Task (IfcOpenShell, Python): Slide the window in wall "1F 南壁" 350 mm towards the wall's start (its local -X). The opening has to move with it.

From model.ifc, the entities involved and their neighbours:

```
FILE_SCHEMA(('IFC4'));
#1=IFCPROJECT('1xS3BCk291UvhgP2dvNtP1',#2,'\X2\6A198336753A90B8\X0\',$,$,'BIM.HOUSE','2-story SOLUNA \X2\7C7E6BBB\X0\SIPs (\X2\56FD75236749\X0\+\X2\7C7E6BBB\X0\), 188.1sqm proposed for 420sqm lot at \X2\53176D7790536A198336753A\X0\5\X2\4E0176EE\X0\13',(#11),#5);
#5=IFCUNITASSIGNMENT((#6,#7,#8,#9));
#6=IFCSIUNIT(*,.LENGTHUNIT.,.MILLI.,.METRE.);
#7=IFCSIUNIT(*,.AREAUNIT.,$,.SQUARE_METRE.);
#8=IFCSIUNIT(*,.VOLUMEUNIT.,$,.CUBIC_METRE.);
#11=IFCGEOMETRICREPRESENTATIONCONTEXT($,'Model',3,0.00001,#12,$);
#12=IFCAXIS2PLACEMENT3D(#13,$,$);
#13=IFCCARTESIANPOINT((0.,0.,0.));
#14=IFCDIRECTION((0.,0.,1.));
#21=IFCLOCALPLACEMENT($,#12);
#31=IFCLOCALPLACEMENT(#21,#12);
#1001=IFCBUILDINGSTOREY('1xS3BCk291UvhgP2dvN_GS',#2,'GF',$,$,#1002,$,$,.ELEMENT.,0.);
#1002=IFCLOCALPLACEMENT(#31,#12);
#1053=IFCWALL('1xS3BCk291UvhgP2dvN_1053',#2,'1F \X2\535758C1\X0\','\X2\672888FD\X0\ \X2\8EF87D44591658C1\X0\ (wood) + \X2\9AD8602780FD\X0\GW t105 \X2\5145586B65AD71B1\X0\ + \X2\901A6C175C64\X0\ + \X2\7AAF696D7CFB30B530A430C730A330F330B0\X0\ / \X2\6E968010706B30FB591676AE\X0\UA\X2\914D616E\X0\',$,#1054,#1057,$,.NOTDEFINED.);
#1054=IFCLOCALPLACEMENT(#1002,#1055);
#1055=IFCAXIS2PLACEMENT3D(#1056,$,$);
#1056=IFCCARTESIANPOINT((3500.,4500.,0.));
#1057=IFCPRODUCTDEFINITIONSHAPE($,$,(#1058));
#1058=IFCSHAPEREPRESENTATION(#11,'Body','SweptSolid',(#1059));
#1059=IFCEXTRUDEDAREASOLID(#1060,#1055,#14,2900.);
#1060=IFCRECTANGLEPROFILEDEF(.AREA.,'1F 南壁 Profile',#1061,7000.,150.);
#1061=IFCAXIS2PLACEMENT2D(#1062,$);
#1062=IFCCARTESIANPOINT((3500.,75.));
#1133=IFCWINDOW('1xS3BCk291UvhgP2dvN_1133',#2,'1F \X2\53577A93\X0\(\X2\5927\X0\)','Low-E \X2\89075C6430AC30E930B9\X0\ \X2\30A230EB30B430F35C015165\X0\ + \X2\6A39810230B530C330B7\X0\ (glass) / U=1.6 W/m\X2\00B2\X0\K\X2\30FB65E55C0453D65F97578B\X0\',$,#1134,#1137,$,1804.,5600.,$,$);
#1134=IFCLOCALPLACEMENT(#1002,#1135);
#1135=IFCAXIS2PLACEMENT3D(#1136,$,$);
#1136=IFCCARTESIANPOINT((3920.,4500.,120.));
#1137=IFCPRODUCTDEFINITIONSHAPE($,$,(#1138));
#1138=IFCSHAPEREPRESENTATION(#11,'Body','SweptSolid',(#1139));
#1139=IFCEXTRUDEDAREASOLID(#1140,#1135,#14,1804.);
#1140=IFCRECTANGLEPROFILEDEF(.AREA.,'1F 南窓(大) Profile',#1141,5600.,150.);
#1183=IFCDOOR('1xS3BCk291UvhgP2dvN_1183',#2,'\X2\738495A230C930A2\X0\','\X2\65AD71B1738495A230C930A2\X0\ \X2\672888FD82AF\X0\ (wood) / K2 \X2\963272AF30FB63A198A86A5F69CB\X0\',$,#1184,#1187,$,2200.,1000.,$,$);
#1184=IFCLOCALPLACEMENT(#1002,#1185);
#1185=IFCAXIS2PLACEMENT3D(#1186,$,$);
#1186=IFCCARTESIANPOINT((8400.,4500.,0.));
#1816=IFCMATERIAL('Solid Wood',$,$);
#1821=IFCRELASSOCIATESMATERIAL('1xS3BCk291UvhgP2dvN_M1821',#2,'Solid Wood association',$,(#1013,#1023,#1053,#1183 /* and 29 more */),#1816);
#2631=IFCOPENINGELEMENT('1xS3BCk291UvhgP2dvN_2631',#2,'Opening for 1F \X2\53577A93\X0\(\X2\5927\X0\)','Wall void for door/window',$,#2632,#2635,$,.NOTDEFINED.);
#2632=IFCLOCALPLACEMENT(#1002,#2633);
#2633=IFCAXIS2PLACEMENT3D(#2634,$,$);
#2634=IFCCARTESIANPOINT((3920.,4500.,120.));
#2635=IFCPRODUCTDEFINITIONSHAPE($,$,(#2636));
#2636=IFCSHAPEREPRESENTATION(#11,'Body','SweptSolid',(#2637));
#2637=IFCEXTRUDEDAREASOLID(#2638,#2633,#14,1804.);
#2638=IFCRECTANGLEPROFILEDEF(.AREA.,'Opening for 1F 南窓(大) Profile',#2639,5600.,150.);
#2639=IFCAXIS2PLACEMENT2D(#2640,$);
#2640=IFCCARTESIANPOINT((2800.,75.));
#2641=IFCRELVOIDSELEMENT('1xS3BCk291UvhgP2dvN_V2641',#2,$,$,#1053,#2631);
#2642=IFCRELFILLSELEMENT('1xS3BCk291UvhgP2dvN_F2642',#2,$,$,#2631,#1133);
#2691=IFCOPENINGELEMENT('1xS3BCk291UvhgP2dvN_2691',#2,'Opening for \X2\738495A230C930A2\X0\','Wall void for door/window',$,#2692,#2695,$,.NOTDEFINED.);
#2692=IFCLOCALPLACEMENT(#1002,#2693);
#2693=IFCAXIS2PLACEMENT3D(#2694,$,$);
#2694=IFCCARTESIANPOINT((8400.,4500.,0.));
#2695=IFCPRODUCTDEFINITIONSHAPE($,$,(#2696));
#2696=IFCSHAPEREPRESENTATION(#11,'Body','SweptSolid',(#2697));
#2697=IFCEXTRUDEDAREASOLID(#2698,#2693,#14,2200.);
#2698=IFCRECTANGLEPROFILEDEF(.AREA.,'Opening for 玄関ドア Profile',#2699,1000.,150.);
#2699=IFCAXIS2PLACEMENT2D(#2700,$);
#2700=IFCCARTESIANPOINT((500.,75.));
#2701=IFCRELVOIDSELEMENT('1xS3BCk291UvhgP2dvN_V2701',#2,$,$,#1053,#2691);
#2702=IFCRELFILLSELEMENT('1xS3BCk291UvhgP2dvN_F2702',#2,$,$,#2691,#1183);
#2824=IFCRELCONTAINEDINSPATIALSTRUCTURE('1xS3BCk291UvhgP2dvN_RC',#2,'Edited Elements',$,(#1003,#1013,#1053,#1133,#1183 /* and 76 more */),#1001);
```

```python
import ifcopenshell
import ifcopenshell.api.geometry
import ifcopenshell.util.placement
import ifcopenshell.util.unit

model = ifcopenshell.open("model.ifc")
unit_scale = ifcopenshell.util.unit.calculate_unit_scale(model)

window = model.by_guid("1xS3BCk291UvhgP2dvN_1133")
opening = window.FillsVoids[0].RelatingOpeningElement
wall = opening.VoidsElements[0].RelatingBuildingElement

wall_matrix = ifcopenshell.util.placement.get_local_placement(wall.ObjectPlacement)
shift = wall_matrix[:3, 0] * -0.35 / unit_scale
before = ifcopenshell.util.placement.get_local_placement(window.ObjectPlacement)[:3, 3].copy()

# The window is not placed relative to its opening, so move both.
for product in (opening, window):
    matrix = ifcopenshell.util.placement.get_local_placement(product.ObjectPlacement)
    matrix[:3, 3] += shift
    ifcopenshell.api.geometry.edit_object_placement(model, product=product, matrix=matrix, is_si=False)

after = ifcopenshell.util.placement.get_local_placement(window.ObjectPlacement)[:3, 3]
print("window moved by", (after - before).round(3) + 0.0)

model.write("model_edited.ifc")
```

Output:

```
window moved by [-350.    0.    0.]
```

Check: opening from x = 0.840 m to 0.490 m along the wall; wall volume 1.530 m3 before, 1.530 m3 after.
